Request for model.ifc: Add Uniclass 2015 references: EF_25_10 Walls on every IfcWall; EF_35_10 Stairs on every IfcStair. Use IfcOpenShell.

First a look at what the model holds.

```python
import ifcopenshell

model = ifcopenshell.open("model.ifc")
print(model.schema)
print("classifications:", [c.Name for c in model.by_type("IfcClassification")])
for ifc_class in ("IfcDoor", "IfcRoof", "IfcStair", "IfcWall", "IfcWindow"):
    print(ifc_class, len(model.by_type(ifc_class)))
```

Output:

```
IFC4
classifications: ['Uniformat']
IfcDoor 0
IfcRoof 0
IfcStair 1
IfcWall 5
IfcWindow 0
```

```python
import ifcopenshell
import ifcopenshell.api.classification

model = ifcopenshell.open("model.ifc")

system = ifcopenshell.api.classification.add_classification(model, classification="Uniclass 2015")

codes = {
    "IfcWall": ("EF_25_10", "Walls"),
    "IfcStair": ("EF_35_10", "Stairs"),
}
for ifc_class, (code, name) in codes.items():
    products = model.by_type(ifc_class)
    ifcopenshell.api.classification.add_reference(
        model, products=products, classification=system, identification=code, name=name
    )
    print(code, len(products))

model.write("model_updated.ifc")
```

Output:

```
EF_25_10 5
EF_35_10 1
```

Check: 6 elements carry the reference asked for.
